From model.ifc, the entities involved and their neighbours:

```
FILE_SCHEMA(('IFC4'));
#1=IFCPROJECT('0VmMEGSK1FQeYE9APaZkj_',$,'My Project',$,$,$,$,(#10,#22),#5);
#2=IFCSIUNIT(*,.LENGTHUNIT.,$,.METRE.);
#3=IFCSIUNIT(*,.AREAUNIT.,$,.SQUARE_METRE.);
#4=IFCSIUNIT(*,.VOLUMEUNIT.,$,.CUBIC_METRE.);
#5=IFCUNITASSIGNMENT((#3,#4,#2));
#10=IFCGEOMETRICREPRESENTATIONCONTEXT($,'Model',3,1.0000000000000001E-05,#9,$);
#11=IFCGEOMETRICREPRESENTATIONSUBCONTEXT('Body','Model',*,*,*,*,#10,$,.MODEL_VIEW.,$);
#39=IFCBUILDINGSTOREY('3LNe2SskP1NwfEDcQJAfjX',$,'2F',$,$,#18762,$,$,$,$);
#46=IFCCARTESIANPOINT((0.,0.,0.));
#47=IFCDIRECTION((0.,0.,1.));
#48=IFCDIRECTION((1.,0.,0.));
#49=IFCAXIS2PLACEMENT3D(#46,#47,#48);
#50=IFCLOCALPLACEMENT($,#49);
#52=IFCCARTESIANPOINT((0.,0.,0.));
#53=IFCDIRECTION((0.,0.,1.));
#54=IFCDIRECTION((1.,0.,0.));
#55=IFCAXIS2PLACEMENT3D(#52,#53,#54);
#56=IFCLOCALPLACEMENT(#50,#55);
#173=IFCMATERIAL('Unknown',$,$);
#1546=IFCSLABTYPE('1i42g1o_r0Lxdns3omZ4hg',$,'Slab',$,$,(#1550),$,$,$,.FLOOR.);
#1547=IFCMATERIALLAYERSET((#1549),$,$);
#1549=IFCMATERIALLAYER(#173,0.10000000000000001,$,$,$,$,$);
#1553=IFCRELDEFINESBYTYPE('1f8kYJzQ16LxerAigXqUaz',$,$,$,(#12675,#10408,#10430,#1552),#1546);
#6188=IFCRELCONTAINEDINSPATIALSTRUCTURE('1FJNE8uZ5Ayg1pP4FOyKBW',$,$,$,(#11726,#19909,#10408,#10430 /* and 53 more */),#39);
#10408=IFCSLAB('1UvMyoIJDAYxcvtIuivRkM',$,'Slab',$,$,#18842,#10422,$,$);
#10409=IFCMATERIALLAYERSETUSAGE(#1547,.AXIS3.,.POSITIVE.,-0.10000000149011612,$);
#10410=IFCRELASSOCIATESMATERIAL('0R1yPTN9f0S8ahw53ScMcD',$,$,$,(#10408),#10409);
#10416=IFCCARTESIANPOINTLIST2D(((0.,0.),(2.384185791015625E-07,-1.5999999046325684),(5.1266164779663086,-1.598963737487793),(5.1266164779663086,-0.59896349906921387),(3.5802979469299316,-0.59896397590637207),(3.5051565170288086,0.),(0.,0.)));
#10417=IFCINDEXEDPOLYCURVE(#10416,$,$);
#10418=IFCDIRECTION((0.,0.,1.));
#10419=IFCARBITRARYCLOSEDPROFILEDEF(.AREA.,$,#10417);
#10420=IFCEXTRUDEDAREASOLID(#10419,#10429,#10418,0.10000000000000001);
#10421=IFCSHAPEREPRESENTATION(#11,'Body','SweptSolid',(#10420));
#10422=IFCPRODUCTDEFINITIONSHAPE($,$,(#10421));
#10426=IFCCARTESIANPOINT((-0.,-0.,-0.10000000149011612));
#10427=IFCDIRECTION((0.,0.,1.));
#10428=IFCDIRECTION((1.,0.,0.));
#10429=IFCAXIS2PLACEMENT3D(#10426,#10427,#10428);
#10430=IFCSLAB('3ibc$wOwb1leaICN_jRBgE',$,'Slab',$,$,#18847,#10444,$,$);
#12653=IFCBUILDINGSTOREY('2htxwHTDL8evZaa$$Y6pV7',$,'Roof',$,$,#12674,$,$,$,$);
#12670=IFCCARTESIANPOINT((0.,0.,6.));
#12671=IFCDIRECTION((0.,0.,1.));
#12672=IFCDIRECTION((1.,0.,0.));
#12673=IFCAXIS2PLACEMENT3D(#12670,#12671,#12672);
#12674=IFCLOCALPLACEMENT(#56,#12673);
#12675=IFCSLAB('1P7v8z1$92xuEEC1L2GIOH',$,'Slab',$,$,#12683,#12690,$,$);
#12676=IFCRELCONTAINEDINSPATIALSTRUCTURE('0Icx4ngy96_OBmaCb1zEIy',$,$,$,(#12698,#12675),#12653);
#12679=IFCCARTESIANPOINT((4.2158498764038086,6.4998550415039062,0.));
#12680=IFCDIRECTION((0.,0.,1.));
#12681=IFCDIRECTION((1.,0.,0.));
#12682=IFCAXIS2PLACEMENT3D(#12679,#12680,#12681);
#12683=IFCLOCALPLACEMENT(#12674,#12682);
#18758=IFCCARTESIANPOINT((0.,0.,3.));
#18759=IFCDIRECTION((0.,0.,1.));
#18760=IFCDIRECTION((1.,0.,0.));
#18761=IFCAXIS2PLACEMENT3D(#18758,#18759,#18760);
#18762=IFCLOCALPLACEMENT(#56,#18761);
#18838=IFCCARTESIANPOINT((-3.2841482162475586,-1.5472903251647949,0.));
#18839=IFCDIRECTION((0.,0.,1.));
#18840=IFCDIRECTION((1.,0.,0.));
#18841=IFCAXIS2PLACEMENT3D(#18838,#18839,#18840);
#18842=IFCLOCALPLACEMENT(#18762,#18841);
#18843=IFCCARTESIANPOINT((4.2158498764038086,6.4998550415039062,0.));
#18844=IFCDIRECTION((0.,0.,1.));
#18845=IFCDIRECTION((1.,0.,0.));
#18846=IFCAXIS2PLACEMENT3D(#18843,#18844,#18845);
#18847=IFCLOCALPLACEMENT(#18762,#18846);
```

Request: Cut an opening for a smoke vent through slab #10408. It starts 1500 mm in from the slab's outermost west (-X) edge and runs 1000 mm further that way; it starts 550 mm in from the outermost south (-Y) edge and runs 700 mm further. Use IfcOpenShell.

```python
import numpy as np
import ifcopenshell
import ifcopenshell.api.feature
import ifcopenshell.api.geometry
import ifcopenshell.api.root
import ifcopenshell.geom
import ifcopenshell.util.placement
import ifcopenshell.util.representation
import ifcopenshell.util.shape
import ifcopenshell.util.unit

model = ifcopenshell.open("model.ifc")
unit_scale = ifcopenshell.util.unit.calculate_unit_scale(model)
settings = ifcopenshell.geom.settings()


def volume(element):
    """Net volume in cubic metres, openings subtracted."""
    shape = ifcopenshell.geom.create_shape(settings, element)
    return ifcopenshell.util.shape.get_volume(shape.geometry)


slab = model.by_guid("1UvMyoIJDAYxcvtIuivRkM")
before = volume(slab)

# Extent in the slab's own axes, in metres. The edges named are its -X and -Y sides.
slab_shape = ifcopenshell.geom.create_shape(settings, slab)
vertices = ifcopenshell.util.shape.get_vertices(slab_shape.geometry)
x_min, y_min, bottom = vertices.min(axis=0)
top = vertices[:, 2].max()

opening = ifcopenshell.api.root.create_entity(model, ifc_class="IfcOpeningElement", name="Smoke vent opening", predefined_type="OPENING")
context = ifcopenshell.util.representation.get_context(model, "Model", "Body", "MODEL_VIEW")
width, depth = 1, 0.7
outline = [(0.0, 0.0), (width, 0.0), (width, depth), (0.0, depth), (0.0, 0.0)]
# Overshoot both faces by 50 mm so the cut is clean.
shape = ifcopenshell.api.geometry.add_slab_representation(
    model, context=context, depth=top - bottom + 0.1, polyline=outline
)
ifcopenshell.api.geometry.assign_representation(model, product=opening, representation=shape)

matrix = ifcopenshell.util.placement.get_local_placement(slab.ObjectPlacement)
matrix[:, 3] = matrix @ np.append(np.array([x_min + 1.5, y_min + 0.55, bottom - 0.05]) / unit_scale, 1.0)
ifcopenshell.api.geometry.edit_object_placement(model, product=opening, matrix=matrix, is_si=False)
ifcopenshell.api.feature.add_feature(model, feature=opening, element=slab)

after = volume(slab)

print(f"slab volume {before:.3f} -> {after:.3f} m3")

model.write("model_rev.ifc")
```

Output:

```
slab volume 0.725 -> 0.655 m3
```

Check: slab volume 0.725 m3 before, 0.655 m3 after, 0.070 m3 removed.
